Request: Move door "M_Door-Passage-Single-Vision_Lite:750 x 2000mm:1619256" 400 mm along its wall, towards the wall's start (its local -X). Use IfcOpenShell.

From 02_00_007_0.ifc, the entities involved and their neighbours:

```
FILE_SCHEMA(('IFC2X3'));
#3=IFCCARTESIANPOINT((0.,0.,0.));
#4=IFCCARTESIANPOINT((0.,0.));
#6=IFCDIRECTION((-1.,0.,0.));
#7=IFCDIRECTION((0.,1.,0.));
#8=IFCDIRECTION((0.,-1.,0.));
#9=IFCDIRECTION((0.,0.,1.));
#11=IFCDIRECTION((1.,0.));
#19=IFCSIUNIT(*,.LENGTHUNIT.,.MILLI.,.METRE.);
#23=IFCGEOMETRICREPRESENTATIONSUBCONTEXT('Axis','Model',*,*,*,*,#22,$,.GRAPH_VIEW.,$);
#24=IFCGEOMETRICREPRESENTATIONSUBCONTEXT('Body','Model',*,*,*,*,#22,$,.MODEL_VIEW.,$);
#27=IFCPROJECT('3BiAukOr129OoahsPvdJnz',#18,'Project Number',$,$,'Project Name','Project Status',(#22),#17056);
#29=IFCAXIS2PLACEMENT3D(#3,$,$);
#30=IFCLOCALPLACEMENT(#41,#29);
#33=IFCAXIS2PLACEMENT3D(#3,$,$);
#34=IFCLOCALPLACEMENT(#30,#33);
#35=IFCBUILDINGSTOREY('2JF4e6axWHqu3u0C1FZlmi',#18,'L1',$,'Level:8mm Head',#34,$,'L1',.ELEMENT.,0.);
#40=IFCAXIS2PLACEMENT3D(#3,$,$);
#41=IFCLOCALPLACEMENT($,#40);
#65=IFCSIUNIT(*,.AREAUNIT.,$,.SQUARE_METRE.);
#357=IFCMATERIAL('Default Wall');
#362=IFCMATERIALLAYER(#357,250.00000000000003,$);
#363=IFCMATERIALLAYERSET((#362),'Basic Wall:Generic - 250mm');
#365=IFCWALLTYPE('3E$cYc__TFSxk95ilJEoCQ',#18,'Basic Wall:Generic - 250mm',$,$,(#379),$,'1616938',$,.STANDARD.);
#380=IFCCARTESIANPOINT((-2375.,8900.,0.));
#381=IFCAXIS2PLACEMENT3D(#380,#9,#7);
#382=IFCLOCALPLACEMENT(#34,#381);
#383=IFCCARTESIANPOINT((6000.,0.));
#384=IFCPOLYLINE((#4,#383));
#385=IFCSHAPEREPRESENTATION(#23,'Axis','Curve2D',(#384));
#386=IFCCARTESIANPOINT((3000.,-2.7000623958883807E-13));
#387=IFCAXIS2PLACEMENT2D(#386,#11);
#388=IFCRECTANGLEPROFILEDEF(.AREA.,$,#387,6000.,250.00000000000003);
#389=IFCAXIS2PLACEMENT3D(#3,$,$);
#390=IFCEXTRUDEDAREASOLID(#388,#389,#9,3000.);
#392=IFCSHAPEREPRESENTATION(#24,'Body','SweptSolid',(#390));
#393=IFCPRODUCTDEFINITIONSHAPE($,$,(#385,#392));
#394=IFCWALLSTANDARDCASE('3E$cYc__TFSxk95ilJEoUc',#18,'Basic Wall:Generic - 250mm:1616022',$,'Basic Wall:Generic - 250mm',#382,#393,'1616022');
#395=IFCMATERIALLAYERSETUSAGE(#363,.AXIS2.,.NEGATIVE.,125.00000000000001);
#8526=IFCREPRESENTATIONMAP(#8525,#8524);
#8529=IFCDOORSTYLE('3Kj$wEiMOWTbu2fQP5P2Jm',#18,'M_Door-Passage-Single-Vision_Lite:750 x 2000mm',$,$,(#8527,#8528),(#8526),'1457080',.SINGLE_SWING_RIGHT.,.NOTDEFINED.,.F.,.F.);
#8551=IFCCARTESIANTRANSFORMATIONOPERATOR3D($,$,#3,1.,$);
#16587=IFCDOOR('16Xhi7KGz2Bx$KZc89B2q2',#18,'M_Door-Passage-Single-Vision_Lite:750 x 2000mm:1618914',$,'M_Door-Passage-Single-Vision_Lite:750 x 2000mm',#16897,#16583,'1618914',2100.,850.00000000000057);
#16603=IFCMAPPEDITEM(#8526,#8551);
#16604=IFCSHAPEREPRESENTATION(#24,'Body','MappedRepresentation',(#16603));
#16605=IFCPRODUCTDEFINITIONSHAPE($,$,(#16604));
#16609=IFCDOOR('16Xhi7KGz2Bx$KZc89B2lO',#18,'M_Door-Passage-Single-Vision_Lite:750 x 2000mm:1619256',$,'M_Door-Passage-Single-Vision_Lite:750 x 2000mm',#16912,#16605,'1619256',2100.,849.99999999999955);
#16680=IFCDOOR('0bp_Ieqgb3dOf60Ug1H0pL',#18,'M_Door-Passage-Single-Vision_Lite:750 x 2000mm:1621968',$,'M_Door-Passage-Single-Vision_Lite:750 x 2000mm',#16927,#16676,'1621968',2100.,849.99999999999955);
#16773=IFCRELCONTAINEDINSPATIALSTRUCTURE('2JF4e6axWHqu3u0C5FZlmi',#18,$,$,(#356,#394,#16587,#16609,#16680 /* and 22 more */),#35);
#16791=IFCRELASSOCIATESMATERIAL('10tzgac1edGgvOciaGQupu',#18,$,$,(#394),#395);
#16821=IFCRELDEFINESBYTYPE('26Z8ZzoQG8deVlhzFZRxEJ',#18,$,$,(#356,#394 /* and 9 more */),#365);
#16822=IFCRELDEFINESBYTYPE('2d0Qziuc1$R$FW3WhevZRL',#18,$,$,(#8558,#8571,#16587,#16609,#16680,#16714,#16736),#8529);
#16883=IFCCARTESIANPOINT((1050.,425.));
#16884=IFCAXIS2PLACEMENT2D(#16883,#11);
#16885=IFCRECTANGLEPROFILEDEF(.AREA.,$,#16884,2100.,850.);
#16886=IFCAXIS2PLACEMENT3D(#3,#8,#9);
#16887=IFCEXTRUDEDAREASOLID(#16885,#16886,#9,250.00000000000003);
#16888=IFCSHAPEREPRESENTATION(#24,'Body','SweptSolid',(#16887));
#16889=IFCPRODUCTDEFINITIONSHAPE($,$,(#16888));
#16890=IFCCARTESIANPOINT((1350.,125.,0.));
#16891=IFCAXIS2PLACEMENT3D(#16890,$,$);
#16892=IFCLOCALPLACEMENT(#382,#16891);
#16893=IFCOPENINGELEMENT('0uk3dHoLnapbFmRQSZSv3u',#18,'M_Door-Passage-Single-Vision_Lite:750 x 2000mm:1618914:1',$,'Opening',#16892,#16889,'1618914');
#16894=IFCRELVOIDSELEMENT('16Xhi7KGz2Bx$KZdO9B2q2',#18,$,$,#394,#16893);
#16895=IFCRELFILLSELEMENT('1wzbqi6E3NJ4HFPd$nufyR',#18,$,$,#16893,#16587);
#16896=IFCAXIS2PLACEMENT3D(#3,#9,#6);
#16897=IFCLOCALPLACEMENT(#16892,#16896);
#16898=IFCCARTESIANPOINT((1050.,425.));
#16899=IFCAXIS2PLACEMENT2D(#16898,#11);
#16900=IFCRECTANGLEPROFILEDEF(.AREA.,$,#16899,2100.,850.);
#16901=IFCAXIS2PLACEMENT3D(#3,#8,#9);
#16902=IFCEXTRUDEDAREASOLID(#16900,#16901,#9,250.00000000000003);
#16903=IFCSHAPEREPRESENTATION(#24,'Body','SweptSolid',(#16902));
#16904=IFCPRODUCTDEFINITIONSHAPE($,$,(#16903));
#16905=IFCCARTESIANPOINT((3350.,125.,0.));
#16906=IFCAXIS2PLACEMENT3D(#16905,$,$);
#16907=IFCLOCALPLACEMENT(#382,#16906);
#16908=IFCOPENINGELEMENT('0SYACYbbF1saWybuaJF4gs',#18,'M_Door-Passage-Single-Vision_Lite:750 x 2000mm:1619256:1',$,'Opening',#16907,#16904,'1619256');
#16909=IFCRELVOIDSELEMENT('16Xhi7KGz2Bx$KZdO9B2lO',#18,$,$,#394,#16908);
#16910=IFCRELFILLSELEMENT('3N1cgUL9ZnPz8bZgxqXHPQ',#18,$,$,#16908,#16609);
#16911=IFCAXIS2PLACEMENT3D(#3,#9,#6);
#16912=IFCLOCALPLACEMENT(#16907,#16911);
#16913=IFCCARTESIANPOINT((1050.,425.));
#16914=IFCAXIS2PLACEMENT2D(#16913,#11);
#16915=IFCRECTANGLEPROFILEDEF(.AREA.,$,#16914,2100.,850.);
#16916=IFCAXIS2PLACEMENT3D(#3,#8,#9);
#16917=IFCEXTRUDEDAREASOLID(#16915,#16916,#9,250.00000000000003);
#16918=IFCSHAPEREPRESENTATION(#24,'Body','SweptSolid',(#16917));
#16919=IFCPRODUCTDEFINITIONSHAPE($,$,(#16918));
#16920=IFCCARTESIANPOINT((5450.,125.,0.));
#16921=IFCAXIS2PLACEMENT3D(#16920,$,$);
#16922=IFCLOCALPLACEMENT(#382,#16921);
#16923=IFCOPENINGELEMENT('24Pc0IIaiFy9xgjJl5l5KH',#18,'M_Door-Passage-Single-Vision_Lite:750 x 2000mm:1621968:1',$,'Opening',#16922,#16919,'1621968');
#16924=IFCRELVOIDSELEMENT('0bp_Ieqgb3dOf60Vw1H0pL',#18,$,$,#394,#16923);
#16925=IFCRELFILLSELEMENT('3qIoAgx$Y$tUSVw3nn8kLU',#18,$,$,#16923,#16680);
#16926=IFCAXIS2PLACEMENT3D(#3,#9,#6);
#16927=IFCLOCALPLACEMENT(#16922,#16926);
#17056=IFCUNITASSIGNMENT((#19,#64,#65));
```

```python
import ifcopenshell
import ifcopenshell.api.geometry
import ifcopenshell.util.placement
import ifcopenshell.util.unit

model = ifcopenshell.open("02_00_007_0.ifc")
unit_scale = ifcopenshell.util.unit.calculate_unit_scale(model)

door = model.by_guid("16Xhi7KGz2Bx$KZc89B2lO")
opening = door.FillsVoids[0].RelatingOpeningElement
wall = opening.VoidsElements[0].RelatingBuildingElement

wall_matrix = ifcopenshell.util.placement.get_local_placement(wall.ObjectPlacement)
shift = wall_matrix[:3, 0] * -0.4 / unit_scale
before = ifcopenshell.util.placement.get_local_placement(door.ObjectPlacement)[:3, 3].copy()

# The door is placed relative to its opening, so it follows when the opening moves.
matrix = ifcopenshell.util.placement.get_local_placement(opening.ObjectPlacement)
matrix[:3, 3] += shift
ifcopenshell.api.geometry.edit_object_placement(
    model, product=opening, matrix=matrix, is_si=False, should_transform_children=True
)

after = ifcopenshell.util.placement.get_local_placement(door.ObjectPlacement)[:3, 3]
print("door moved by", (after - before).round(3) + 0.0)

model.write("02_00_007_0_updated.ifc")
```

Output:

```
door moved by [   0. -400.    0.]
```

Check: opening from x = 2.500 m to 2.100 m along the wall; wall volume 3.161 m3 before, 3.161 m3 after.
